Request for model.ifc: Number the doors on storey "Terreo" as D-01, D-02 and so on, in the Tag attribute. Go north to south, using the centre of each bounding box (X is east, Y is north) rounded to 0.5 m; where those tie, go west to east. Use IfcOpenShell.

First a look at what the model holds.

```python
import ifcopenshell
import ifcopenshell.util.element
import ifcopenshell.util.placement

model = ifcopenshell.open("model.ifc")
print(model.schema)
storey = next(s for s in model.by_type("IfcBuildingStorey") if s.Name == "Terreo")
doors = [e for e in ifcopenshell.util.element.get_decomposition(storey) if e.is_a("IfcDoor")]
for e in sorted(doors, key=lambda e: e.id()):
    origin = ifcopenshell.util.placement.get_local_placement(e.ObjectPlacement)[:3, 3]
    print(e.id(), e.Tag, e.Name, origin.round(2) + 0.0, sep=" | ")
```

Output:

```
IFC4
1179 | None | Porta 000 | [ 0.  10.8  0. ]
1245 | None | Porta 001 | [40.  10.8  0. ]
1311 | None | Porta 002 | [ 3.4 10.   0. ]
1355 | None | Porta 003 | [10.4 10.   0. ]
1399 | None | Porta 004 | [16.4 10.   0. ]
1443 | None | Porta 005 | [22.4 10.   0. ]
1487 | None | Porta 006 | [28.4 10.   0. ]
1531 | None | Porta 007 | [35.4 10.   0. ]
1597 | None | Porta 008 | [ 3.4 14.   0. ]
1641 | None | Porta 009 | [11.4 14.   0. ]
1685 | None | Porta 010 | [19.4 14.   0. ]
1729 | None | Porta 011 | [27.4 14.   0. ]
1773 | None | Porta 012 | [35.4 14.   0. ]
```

```python
import ifcopenshell
import ifcopenshell.geom
import ifcopenshell.util.element
import ifcopenshell.util.shape

model = ifcopenshell.open("model.ifc")
settings = ifcopenshell.geom.settings()
settings.set("use-world-coords", True)


def centre(element):
    shape = ifcopenshell.geom.create_shape(settings, element)
    return ifcopenshell.util.shape.get_bbox_centroid(shape.geometry)


storey = next(s for s in model.by_type("IfcBuildingStorey") if s.Name == "Terreo")
doors = [e for e in ifcopenshell.util.element.get_decomposition(storey) if e.is_a("IfcDoor")]

# Insertion points can sit at a corner or the storey origin, so sort by the geometry (in metres).
centres = {e: centre(e) for e in doors}
doors.sort(key=lambda e: (-round(centres[e][1] / 0.5), centres[e][0]))

for i, e in enumerate(doors, start=1):
    number = f"D-{i:02d}"
    e.Tag = number
    print(e.id(), number)

model.write("model_updated.ifc")
```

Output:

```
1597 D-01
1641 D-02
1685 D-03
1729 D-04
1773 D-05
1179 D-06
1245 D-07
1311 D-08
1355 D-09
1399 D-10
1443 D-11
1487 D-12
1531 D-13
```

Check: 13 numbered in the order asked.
